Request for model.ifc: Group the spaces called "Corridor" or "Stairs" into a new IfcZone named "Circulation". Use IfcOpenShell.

First a look at what the model holds.

```python
import ifcopenshell

model = ifcopenshell.open("model.ifc")
print(model.schema)
seen = {}
for space in model.by_type("IfcSpace"):
    seen[space.LongName] = seen.get(space.LongName, 0) + 1
for name, count in sorted(seen.items(), key=str):
    print(count, "x", name)
print("zones:", [z.Name for z in model.by_type("IfcZone")][:20])
```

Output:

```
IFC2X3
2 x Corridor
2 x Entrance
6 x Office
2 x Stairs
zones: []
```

```python
import ifcopenshell
import ifcopenshell.api.group
import ifcopenshell.api.root

model = ifcopenshell.open("model.ifc")

names = {"Corridor", "Stairs"}
spaces = [s for s in model.by_type("IfcSpace") if s.LongName in names]

zone = ifcopenshell.api.root.create_entity(model, ifc_class="IfcZone", name="Circulation")
ifcopenshell.api.group.assign_group(model, products=spaces, group=zone)
print(len(spaces), "spaces in", zone.Name)

model.write("model_rev.ifc")
```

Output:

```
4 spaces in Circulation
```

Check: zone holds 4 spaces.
